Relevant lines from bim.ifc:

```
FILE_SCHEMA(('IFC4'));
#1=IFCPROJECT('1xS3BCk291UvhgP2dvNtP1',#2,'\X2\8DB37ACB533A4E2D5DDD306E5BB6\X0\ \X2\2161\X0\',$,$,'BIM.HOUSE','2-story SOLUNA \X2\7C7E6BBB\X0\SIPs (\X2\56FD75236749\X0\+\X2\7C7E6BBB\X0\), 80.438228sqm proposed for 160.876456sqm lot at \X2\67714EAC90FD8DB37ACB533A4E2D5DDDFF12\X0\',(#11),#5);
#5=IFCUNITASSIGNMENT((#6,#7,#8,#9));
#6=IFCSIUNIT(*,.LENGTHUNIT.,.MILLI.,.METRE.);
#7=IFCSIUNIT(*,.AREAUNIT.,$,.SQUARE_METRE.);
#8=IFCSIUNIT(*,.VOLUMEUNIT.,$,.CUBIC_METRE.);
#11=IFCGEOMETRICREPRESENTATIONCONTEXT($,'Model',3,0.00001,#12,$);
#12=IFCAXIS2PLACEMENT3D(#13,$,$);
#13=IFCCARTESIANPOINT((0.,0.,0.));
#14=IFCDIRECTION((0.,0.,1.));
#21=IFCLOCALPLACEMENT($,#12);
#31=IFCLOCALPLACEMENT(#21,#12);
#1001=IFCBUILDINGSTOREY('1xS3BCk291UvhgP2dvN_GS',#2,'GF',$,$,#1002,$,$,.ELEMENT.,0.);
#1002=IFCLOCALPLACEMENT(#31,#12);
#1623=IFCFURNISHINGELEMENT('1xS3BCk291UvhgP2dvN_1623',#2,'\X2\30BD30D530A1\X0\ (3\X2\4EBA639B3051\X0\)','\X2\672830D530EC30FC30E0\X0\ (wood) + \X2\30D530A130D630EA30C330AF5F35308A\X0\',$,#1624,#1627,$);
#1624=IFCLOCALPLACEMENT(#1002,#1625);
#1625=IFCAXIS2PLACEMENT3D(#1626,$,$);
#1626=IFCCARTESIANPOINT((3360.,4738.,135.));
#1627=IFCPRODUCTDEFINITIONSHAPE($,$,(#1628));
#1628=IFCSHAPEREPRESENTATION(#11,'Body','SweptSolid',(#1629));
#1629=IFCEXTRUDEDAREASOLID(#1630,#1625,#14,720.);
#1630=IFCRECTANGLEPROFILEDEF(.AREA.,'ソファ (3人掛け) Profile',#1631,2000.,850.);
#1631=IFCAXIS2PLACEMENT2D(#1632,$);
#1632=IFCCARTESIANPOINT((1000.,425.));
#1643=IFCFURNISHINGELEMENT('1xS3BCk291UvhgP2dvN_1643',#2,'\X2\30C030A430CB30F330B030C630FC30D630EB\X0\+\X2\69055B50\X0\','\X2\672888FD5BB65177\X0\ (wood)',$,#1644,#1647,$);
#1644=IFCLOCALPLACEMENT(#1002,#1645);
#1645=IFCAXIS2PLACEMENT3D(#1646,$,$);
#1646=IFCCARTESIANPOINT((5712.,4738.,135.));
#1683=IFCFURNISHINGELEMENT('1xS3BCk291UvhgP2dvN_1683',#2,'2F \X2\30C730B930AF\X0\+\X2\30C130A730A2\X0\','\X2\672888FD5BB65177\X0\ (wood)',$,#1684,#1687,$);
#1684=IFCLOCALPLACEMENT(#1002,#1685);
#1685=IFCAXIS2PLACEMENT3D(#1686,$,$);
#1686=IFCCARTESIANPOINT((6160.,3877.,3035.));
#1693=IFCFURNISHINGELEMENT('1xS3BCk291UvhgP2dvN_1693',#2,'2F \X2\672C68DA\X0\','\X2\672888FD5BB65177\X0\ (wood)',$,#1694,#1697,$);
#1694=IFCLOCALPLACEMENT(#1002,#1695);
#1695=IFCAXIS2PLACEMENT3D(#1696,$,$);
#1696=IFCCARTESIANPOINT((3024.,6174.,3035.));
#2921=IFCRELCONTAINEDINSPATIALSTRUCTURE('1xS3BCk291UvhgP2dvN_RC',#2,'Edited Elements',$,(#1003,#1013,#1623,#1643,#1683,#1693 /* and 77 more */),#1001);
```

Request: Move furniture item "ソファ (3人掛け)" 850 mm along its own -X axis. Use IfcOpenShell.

```python
import ifcopenshell
import ifcopenshell.api.geometry
import ifcopenshell.util.placement
import ifcopenshell.util.unit

model = ifcopenshell.open("bim.ifc")
unit_scale = ifcopenshell.util.unit.calculate_unit_scale(model)

item = model.by_guid("1xS3BCk291UvhgP2dvN_1623")
matrix = ifcopenshell.util.placement.get_local_placement(item.ObjectPlacement)
matrix[:3, 3] -= matrix[:3, 0] * 0.85 / unit_scale
ifcopenshell.api.geometry.edit_object_placement(model, product=item, matrix=matrix, is_si=False)

print(ifcopenshell.util.placement.get_local_placement(item.ObjectPlacement).round(3) + 0.0)

model.write("bim-out.ifc")
```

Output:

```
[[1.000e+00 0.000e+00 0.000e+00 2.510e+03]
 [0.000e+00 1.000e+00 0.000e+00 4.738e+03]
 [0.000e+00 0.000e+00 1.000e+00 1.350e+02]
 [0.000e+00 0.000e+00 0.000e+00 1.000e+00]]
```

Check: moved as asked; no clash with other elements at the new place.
